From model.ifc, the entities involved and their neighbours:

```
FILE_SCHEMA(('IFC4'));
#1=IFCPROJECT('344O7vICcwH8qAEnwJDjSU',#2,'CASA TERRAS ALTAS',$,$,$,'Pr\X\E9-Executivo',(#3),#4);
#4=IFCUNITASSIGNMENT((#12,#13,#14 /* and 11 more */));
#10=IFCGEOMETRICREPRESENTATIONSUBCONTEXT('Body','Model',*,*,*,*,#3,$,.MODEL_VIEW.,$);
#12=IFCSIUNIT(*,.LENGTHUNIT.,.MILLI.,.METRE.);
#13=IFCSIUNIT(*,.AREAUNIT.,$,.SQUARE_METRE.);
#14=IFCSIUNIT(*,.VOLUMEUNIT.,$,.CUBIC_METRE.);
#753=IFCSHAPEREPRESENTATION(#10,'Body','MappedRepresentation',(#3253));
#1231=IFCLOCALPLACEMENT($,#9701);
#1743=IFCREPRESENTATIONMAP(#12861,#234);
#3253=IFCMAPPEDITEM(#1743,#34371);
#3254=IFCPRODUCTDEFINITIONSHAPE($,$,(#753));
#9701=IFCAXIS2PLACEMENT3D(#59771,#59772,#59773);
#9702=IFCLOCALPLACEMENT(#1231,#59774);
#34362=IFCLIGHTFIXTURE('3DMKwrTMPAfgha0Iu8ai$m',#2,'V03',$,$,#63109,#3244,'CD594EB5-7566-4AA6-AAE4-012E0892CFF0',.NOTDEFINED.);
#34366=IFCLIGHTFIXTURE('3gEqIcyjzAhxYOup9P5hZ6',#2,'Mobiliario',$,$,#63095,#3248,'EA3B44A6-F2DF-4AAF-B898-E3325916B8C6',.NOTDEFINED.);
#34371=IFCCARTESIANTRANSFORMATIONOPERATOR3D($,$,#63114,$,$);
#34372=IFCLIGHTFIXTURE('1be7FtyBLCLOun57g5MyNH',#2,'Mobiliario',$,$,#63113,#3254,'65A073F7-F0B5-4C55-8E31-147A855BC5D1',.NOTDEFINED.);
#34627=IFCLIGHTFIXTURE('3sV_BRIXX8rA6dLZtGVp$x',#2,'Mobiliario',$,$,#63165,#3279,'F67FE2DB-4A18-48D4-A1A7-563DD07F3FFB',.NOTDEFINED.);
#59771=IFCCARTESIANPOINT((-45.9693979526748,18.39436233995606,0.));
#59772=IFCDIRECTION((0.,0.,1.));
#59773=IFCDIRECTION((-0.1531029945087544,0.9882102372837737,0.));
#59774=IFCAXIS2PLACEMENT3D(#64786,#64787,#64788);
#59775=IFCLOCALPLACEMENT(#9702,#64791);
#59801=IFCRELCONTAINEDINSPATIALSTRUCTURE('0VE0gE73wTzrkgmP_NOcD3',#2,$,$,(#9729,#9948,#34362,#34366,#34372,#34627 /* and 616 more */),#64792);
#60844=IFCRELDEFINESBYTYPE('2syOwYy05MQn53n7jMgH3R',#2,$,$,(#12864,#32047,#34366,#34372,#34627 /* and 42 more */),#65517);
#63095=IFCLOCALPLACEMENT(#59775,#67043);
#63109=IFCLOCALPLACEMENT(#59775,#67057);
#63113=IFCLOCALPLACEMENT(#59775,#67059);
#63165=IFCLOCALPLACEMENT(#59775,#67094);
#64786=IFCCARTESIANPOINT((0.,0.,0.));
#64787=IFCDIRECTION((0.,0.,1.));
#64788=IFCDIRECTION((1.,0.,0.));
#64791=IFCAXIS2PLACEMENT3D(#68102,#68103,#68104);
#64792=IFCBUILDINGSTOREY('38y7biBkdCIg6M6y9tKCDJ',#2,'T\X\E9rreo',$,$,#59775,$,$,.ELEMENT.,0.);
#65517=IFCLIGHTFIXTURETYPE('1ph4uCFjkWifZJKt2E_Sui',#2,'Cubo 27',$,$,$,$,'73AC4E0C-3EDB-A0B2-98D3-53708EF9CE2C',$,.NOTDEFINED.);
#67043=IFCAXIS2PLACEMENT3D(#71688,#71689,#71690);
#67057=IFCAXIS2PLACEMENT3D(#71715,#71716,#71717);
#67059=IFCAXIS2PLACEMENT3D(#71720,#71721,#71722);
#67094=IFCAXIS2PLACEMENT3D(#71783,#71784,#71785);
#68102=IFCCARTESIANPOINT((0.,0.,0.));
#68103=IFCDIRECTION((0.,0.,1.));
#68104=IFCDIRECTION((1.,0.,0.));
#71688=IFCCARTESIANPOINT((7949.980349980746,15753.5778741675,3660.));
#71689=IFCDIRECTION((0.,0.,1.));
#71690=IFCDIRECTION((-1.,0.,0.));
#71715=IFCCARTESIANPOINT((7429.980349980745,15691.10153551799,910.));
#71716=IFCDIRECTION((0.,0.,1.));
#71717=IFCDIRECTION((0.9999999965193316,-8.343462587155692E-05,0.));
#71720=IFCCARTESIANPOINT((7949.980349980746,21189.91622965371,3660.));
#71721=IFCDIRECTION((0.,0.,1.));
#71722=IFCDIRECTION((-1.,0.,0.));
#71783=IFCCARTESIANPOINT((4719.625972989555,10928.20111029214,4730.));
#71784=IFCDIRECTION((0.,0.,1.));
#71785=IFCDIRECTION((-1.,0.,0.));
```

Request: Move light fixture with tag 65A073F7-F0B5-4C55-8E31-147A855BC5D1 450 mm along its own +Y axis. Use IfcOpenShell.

```python
import ifcopenshell
import ifcopenshell.api.geometry
import ifcopenshell.util.placement
import ifcopenshell.util.unit

model = ifcopenshell.open("model.ifc")
unit_scale = ifcopenshell.util.unit.calculate_unit_scale(model)

item = model.by_id(34372)
matrix = ifcopenshell.util.placement.get_local_placement(item.ObjectPlacement)
matrix[:3, 3] += matrix[:3, 1] * 0.45 / unit_scale
ifcopenshell.api.geometry.edit_object_placement(model, product=item, matrix=matrix, is_si=False)

print(ifcopenshell.util.placement.get_local_placement(item.ObjectPlacement).round(3) + 0.0)

model.write("model_edited.ifc")
```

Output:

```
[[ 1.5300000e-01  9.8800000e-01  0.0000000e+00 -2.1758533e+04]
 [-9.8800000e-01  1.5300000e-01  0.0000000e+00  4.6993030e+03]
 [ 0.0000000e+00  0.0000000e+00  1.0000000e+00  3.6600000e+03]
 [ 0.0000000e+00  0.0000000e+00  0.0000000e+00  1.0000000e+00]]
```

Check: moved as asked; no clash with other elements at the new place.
